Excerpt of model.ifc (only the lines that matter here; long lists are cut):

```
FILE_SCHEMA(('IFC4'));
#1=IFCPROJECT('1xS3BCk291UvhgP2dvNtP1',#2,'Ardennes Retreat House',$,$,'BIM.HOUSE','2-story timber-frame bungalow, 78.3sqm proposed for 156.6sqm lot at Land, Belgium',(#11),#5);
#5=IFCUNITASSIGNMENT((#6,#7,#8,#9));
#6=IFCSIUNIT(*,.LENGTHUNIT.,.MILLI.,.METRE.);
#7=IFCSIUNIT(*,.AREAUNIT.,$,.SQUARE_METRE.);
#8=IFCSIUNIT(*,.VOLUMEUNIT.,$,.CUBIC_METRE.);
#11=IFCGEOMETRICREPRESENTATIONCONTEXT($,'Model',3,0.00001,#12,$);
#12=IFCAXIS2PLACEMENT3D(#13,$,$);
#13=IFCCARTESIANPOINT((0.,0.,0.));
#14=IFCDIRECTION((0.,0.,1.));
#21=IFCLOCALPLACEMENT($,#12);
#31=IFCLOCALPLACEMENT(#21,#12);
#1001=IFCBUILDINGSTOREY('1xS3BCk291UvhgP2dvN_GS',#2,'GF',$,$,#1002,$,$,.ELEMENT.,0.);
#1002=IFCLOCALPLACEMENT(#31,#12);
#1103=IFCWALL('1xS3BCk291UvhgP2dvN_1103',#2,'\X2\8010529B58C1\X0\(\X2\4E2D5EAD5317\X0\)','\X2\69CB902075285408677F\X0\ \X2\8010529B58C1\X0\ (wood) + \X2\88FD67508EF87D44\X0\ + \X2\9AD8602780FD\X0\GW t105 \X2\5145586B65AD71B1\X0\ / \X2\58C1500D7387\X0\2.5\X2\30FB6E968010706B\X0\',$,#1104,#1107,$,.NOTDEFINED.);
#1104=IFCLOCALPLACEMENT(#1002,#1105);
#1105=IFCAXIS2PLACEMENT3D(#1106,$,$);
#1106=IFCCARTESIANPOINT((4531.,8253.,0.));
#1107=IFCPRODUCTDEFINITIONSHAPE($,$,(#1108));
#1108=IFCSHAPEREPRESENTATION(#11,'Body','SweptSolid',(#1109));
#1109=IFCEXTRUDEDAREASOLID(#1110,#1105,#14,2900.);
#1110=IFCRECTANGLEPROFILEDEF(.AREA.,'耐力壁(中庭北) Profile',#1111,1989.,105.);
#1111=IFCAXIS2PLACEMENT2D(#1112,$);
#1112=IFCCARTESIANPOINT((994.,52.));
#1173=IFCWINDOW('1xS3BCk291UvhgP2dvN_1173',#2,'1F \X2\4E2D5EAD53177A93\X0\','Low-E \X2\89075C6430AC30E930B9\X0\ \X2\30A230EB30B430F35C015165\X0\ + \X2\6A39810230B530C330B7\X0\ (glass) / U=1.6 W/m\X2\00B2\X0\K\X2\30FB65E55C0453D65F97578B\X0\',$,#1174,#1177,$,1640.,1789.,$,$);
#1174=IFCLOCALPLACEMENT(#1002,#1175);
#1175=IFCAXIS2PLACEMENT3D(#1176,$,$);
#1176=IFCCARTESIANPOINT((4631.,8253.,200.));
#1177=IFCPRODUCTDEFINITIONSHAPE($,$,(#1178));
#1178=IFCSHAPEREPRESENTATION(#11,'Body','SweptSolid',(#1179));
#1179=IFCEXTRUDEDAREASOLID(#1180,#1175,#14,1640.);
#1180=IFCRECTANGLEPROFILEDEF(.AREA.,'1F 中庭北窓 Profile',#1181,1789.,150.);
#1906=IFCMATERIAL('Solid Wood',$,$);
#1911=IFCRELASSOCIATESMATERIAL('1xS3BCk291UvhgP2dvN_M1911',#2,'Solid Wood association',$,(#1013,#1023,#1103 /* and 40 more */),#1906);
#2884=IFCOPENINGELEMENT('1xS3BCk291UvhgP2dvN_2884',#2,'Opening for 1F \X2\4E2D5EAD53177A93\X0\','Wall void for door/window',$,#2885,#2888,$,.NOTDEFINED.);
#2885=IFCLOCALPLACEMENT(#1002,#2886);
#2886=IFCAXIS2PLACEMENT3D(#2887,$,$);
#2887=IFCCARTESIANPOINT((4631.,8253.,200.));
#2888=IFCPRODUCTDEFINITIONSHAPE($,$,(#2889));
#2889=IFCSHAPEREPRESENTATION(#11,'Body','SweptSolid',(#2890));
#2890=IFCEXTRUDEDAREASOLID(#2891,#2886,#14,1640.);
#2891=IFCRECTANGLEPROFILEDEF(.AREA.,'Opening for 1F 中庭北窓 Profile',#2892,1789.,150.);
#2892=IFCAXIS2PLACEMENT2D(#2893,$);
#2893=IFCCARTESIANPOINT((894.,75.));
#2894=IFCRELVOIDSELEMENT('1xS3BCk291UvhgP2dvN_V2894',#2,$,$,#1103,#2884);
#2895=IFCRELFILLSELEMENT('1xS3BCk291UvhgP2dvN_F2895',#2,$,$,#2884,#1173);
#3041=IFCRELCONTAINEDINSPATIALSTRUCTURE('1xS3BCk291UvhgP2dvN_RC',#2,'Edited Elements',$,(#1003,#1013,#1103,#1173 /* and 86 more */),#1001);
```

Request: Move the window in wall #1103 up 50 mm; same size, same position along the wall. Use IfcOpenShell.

```python
import numpy as np
import ifcopenshell
import ifcopenshell.api.geometry
import ifcopenshell.util.placement
import ifcopenshell.util.unit

model = ifcopenshell.open("model.ifc")
unit_scale = ifcopenshell.util.unit.calculate_unit_scale(model)

window = model.by_guid("1xS3BCk291UvhgP2dvN_1173")
opening = window.FillsVoids[0].RelatingOpeningElement
dz = 0.05 / unit_scale

shift = np.array([0.0, 0.0, dz])
# The window is not placed relative to its opening, so move both.
for product in (opening, window):
    matrix = ifcopenshell.util.placement.get_local_placement(product.ObjectPlacement)
    matrix[:3, 3] += shift
    ifcopenshell.api.geometry.edit_object_placement(model, product=product, matrix=matrix, is_si=False)

print(f"moved by {dz * unit_scale:+.3f} m")

model.write("model_v2.ifc")
```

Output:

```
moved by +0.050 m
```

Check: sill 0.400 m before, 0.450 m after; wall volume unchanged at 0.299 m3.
